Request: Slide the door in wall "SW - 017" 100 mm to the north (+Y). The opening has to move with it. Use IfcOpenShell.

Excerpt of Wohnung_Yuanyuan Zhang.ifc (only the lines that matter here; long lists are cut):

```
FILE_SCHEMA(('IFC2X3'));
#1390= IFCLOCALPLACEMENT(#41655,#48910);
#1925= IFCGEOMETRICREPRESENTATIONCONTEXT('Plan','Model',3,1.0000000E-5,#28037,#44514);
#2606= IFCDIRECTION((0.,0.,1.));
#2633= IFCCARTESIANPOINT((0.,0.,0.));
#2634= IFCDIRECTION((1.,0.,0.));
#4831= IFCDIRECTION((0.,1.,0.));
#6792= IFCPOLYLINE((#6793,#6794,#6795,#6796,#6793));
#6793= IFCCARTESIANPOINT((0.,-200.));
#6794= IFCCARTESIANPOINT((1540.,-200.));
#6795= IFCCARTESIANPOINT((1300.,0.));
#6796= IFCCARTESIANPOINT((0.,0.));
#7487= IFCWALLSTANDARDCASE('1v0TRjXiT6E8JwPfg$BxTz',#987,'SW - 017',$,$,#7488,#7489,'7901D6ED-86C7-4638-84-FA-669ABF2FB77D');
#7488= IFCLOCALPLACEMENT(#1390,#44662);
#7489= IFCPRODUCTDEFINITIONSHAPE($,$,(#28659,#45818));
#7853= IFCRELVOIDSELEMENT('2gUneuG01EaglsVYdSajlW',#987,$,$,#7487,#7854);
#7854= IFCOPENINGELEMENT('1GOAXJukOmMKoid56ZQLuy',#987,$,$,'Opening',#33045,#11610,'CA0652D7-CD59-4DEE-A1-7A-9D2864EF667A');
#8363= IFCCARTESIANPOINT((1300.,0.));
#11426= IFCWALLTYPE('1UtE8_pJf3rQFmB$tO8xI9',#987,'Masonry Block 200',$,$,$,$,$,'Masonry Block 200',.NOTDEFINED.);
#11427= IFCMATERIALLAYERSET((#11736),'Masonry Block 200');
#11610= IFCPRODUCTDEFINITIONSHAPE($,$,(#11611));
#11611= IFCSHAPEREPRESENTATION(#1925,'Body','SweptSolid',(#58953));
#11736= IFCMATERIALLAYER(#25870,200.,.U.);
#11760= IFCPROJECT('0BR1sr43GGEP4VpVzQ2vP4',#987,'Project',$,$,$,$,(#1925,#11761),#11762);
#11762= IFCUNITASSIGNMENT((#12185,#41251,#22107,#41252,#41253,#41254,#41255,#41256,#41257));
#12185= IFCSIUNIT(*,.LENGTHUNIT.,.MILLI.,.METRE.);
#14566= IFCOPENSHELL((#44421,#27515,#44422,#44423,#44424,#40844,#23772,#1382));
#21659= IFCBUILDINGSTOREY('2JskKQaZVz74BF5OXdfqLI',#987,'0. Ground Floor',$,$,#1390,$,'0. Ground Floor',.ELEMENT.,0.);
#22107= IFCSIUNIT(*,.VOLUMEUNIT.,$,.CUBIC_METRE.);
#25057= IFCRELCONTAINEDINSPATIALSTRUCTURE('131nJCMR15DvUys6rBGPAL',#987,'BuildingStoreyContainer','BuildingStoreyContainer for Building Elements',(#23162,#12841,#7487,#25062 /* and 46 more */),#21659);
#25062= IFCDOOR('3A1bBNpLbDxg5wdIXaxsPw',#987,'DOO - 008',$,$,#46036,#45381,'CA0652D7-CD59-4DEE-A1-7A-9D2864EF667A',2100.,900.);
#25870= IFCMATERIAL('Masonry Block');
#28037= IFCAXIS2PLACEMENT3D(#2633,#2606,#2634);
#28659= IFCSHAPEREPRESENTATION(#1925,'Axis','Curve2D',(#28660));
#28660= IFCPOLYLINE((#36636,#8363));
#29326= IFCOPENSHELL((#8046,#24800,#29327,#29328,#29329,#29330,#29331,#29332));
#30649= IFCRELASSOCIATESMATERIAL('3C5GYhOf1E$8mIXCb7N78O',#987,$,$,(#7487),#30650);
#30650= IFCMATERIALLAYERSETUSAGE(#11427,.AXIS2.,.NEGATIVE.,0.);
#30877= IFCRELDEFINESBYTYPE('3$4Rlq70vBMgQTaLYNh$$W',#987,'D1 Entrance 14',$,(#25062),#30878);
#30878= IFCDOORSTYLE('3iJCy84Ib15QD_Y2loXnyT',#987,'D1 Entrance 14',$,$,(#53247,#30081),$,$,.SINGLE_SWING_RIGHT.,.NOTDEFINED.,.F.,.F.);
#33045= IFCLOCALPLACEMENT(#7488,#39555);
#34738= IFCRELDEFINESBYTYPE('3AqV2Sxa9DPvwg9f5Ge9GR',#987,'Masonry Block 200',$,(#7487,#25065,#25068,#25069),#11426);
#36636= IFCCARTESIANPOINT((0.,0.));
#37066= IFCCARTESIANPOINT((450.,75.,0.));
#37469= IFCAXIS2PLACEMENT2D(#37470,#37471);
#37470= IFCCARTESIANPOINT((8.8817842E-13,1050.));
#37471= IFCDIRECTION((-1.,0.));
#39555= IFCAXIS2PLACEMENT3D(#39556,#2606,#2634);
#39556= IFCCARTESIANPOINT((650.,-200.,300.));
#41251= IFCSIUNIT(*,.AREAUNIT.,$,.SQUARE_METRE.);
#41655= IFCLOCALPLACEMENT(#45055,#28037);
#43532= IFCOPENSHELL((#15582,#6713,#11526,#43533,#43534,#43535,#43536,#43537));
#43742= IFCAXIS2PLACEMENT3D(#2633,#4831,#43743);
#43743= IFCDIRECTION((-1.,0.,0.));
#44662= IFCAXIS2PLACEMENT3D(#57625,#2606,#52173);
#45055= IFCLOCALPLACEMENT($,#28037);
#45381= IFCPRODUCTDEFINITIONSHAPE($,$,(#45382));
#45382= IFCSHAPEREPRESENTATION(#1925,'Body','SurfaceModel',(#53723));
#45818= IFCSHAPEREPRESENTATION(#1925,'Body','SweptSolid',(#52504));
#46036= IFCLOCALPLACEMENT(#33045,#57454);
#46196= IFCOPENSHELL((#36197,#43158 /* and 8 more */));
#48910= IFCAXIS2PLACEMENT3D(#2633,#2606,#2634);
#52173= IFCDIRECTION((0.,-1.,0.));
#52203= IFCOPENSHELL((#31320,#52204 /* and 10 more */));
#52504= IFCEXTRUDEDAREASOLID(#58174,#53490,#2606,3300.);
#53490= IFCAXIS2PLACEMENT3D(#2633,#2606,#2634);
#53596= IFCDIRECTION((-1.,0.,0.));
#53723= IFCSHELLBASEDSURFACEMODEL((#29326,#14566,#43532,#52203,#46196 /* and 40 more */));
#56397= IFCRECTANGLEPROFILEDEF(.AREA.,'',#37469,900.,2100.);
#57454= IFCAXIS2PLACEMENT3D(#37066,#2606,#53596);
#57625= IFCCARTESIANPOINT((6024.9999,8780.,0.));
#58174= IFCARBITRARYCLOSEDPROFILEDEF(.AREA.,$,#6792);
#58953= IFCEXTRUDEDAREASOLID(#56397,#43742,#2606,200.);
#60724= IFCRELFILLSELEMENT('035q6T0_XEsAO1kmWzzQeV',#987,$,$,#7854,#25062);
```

```python
import ifcopenshell
import ifcopenshell.api.geometry
import ifcopenshell.util.placement
import ifcopenshell.util.unit

model = ifcopenshell.open("Wohnung_Yuanyuan Zhang.ifc")
unit_scale = ifcopenshell.util.unit.calculate_unit_scale(model)

door = model.by_guid("3A1bBNpLbDxg5wdIXaxsPw")
opening = door.FillsVoids[0].RelatingOpeningElement
wall = opening.VoidsElements[0].RelatingBuildingElement

wall_matrix = ifcopenshell.util.placement.get_local_placement(wall.ObjectPlacement)
shift = wall_matrix[:3, 0] * -0.1 / unit_scale
before = ifcopenshell.util.placement.get_local_placement(door.ObjectPlacement)[:3, 3].copy()

# The door is placed relative to its opening, so it follows when the opening moves.
matrix = ifcopenshell.util.placement.get_local_placement(opening.ObjectPlacement)
matrix[:3, 3] += shift
ifcopenshell.api.geometry.edit_object_placement(
    model, product=opening, matrix=matrix, is_si=False, should_transform_children=True
)

after = ifcopenshell.util.placement.get_local_placement(door.ObjectPlacement)[:3, 3]
print("door moved by", (after - before).round(3) + 0.0)

model.write("Wohnung_Yuanyuan Zhang-out.ifc")
```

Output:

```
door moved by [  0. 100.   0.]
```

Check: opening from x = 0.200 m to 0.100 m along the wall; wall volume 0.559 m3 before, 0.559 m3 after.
